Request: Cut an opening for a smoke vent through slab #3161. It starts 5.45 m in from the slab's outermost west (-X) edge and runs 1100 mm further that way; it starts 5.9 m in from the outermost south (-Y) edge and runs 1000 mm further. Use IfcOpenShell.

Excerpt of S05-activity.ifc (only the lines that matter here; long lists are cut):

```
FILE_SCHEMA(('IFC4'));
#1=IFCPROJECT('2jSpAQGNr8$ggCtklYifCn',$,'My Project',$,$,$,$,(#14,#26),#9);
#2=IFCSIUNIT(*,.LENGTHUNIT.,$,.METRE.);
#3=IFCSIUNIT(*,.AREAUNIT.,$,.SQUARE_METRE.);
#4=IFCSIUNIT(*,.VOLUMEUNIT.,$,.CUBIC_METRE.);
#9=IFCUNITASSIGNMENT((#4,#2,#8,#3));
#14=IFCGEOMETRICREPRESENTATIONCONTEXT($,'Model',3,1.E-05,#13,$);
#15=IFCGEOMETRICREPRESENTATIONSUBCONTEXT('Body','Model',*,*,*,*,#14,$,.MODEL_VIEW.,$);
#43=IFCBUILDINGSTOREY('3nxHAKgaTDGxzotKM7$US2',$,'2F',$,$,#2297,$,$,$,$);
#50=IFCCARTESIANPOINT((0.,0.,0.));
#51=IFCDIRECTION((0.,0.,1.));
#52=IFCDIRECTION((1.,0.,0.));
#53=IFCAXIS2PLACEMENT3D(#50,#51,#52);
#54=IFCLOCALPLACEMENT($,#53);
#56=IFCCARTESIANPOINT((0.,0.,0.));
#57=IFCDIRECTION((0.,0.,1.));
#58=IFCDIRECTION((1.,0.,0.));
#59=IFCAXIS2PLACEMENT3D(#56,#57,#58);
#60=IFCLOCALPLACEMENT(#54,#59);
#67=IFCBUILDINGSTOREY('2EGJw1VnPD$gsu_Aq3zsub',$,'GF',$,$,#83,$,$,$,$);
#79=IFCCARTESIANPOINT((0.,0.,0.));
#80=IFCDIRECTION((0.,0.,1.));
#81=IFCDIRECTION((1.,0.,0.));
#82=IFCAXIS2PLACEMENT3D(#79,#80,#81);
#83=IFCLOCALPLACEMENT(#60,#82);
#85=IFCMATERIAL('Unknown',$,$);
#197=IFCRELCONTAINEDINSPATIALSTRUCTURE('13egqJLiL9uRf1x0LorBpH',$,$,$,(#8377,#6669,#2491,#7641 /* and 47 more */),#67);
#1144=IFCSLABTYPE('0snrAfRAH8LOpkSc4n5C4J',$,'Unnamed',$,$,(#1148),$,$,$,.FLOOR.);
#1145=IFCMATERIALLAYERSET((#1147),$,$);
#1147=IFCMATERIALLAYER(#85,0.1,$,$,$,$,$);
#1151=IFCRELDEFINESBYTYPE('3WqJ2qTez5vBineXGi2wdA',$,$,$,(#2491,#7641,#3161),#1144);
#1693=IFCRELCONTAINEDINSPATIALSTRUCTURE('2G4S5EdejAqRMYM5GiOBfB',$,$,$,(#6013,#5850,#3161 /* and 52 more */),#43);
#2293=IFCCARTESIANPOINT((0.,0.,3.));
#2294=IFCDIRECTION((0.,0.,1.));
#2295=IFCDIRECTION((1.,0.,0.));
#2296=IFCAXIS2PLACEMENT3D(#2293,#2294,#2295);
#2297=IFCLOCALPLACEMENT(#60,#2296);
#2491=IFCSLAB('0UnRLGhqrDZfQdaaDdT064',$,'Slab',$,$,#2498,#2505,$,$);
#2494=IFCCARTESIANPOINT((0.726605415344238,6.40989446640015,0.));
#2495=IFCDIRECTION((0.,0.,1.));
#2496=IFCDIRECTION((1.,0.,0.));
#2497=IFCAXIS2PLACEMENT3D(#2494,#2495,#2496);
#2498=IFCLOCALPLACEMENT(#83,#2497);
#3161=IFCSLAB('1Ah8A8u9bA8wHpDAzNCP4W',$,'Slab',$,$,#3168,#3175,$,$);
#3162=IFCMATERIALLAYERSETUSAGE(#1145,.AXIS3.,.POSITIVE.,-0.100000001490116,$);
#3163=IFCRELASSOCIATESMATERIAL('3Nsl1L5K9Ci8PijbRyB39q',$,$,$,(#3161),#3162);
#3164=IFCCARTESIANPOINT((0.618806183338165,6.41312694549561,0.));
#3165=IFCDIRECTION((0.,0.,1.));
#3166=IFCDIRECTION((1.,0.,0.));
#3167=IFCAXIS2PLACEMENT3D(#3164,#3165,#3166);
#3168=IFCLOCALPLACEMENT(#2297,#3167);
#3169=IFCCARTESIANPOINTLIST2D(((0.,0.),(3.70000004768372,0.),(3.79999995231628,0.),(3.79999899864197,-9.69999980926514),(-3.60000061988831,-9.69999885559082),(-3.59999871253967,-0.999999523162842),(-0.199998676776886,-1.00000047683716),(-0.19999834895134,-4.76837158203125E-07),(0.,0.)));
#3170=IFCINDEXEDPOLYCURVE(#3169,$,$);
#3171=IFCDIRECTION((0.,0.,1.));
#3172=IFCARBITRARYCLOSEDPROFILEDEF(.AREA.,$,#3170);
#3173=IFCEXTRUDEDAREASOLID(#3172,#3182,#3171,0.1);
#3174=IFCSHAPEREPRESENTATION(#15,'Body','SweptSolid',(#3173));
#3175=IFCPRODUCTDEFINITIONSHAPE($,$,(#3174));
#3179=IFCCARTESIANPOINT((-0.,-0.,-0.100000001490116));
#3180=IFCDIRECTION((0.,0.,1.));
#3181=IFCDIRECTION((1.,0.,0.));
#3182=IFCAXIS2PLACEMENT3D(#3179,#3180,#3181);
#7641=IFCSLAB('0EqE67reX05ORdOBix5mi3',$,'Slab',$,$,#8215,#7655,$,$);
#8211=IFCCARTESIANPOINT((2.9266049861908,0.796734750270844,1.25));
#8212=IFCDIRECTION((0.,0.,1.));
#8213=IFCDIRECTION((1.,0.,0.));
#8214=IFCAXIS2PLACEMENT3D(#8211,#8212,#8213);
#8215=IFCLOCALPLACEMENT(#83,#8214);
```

```python
import numpy as np
import ifcopenshell
import ifcopenshell.api.feature
import ifcopenshell.api.geometry
import ifcopenshell.api.root
import ifcopenshell.geom
import ifcopenshell.util.placement
import ifcopenshell.util.representation
import ifcopenshell.util.shape
import ifcopenshell.util.unit

model = ifcopenshell.open("S05-activity.ifc")
unit_scale = ifcopenshell.util.unit.calculate_unit_scale(model)
settings = ifcopenshell.geom.settings()


def volume(element):
    """Net volume in cubic metres, openings subtracted."""
    shape = ifcopenshell.geom.create_shape(settings, element)
    return ifcopenshell.util.shape.get_volume(shape.geometry)


slab = model.by_guid("1Ah8A8u9bA8wHpDAzNCP4W")
before = volume(slab)

# Extent in the slab's own axes, in metres. The edges named are its -X and -Y sides.
slab_shape = ifcopenshell.geom.create_shape(settings, slab)
vertices = ifcopenshell.util.shape.get_vertices(slab_shape.geometry)
x_min, y_min, bottom = vertices.min(axis=0)
top = vertices[:, 2].max()

opening = ifcopenshell.api.root.create_entity(model, ifc_class="IfcOpeningElement", name="Smoke vent opening", predefined_type="OPENING")
context = ifcopenshell.util.representation.get_context(model, "Model", "Body", "MODEL_VIEW")
width, depth = 1.1, 1
outline = [(0.0, 0.0), (width, 0.0), (width, depth), (0.0, depth), (0.0, 0.0)]
# Overshoot both faces by 50 mm so the cut is clean.
shape = ifcopenshell.api.geometry.add_slab_representation(
    model, context=context, depth=top - bottom + 0.1, polyline=outline
)
ifcopenshell.api.geometry.assign_representation(model, product=opening, representation=shape)

matrix = ifcopenshell.util.placement.get_local_placement(slab.ObjectPlacement)
matrix[:, 3] = matrix @ np.append(np.array([x_min + 5.45, y_min + 5.9, bottom - 0.05]) / unit_scale, 1.0)
ifcopenshell.api.geometry.edit_object_placement(model, product=opening, matrix=matrix, is_si=False)
ifcopenshell.api.feature.add_feature(model, feature=opening, element=slab)

after = volume(slab)

print(f"slab volume {before:.3f} -> {after:.3f} m3")

model.write("S05-activity_updated.ifc")
```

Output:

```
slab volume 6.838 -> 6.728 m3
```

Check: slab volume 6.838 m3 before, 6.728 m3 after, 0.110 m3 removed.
